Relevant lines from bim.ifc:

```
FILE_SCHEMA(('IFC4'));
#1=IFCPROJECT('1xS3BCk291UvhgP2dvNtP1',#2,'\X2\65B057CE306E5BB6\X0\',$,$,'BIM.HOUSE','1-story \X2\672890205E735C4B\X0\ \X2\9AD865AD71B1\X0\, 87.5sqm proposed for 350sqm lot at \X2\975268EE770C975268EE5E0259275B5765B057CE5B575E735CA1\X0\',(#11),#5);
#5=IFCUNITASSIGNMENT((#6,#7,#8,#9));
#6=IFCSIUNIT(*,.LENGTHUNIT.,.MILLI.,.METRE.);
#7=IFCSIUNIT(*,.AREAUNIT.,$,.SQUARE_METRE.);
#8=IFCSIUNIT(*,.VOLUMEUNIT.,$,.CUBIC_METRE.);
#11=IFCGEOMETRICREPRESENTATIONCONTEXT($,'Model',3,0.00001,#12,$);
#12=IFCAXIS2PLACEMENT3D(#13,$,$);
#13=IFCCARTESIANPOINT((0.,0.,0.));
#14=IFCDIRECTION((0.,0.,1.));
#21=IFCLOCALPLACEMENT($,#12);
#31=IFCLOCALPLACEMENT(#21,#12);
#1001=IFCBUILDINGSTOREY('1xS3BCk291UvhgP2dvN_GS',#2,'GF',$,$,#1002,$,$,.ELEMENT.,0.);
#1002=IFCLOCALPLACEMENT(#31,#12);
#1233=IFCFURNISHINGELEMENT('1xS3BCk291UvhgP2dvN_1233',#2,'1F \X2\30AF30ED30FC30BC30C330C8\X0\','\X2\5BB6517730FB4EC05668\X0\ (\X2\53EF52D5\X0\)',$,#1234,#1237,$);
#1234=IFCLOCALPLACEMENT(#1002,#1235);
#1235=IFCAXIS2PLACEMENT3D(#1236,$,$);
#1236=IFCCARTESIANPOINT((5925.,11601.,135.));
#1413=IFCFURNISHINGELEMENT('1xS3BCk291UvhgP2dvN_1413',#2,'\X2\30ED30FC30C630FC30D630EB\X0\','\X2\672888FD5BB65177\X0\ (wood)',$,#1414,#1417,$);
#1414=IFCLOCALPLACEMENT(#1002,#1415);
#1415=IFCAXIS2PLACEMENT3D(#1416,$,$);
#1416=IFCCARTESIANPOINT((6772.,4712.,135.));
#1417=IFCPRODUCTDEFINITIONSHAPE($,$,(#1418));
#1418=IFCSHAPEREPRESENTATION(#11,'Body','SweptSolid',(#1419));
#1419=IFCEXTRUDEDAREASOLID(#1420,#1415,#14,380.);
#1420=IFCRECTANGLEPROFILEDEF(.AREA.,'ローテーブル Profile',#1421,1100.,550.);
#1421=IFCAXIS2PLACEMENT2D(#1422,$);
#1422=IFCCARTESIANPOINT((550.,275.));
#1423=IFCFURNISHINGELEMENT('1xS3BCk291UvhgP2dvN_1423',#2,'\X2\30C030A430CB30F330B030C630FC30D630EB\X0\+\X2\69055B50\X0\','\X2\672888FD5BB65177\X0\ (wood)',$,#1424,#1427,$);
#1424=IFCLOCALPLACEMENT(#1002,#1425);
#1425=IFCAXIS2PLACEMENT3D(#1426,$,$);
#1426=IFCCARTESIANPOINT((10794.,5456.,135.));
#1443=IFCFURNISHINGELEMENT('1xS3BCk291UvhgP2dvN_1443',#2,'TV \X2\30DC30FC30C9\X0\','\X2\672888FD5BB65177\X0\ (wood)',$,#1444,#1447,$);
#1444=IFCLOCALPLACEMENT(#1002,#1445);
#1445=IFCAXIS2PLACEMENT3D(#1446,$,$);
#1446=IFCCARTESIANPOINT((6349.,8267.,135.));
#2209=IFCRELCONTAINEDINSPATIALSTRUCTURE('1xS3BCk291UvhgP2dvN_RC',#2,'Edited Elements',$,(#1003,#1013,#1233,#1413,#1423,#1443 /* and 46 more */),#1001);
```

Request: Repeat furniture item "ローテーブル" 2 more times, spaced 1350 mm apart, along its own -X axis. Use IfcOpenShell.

```python
import ifcopenshell
import ifcopenshell.api.geometry
import ifcopenshell.api.root
import ifcopenshell.util.element
import ifcopenshell.util.placement
import ifcopenshell.util.unit

model = ifcopenshell.open("bim.ifc")
unit_scale = ifcopenshell.util.unit.calculate_unit_scale(model)


def reuse_history(source, copy):
    """copy_class also copies each property set's owner history, people and application; keep the originals."""
    for rel in copy.IsDefinedBy:
        if rel.is_a("IfcRelDefinesByProperties") and (history := rel.RelatingPropertyDefinition.OwnerHistory):
            rel.RelatingPropertyDefinition.OwnerHistory = source.OwnerHistory
            ifcopenshell.util.element.remove_deep2(model, history)


source = model.by_guid("1xS3BCk291UvhgP2dvN_1413")
base = ifcopenshell.util.placement.get_local_placement(source.ObjectPlacement)
step = -base[:3, 0] * 1.35 / unit_scale

for i in range(1, 3):
    copy = ifcopenshell.api.root.copy_class(model, product=source)
    copy.Representation = ifcopenshell.util.element.copy_deep(
        model, source.Representation, exclude=["IfcGeometricRepresentationContext", "IfcRepresentationMap"]
    )
    reuse_history(source, copy)
    matrix = base.copy()
    matrix[:3, 3] += i * step
    print("added at", matrix[:3, 3].round(3) + 0.0)
    ifcopenshell.api.geometry.edit_object_placement(model, product=copy, matrix=matrix, is_si=False)

model.write("bim_updated.ifc")
```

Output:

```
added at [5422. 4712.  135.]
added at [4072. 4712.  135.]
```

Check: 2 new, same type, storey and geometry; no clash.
